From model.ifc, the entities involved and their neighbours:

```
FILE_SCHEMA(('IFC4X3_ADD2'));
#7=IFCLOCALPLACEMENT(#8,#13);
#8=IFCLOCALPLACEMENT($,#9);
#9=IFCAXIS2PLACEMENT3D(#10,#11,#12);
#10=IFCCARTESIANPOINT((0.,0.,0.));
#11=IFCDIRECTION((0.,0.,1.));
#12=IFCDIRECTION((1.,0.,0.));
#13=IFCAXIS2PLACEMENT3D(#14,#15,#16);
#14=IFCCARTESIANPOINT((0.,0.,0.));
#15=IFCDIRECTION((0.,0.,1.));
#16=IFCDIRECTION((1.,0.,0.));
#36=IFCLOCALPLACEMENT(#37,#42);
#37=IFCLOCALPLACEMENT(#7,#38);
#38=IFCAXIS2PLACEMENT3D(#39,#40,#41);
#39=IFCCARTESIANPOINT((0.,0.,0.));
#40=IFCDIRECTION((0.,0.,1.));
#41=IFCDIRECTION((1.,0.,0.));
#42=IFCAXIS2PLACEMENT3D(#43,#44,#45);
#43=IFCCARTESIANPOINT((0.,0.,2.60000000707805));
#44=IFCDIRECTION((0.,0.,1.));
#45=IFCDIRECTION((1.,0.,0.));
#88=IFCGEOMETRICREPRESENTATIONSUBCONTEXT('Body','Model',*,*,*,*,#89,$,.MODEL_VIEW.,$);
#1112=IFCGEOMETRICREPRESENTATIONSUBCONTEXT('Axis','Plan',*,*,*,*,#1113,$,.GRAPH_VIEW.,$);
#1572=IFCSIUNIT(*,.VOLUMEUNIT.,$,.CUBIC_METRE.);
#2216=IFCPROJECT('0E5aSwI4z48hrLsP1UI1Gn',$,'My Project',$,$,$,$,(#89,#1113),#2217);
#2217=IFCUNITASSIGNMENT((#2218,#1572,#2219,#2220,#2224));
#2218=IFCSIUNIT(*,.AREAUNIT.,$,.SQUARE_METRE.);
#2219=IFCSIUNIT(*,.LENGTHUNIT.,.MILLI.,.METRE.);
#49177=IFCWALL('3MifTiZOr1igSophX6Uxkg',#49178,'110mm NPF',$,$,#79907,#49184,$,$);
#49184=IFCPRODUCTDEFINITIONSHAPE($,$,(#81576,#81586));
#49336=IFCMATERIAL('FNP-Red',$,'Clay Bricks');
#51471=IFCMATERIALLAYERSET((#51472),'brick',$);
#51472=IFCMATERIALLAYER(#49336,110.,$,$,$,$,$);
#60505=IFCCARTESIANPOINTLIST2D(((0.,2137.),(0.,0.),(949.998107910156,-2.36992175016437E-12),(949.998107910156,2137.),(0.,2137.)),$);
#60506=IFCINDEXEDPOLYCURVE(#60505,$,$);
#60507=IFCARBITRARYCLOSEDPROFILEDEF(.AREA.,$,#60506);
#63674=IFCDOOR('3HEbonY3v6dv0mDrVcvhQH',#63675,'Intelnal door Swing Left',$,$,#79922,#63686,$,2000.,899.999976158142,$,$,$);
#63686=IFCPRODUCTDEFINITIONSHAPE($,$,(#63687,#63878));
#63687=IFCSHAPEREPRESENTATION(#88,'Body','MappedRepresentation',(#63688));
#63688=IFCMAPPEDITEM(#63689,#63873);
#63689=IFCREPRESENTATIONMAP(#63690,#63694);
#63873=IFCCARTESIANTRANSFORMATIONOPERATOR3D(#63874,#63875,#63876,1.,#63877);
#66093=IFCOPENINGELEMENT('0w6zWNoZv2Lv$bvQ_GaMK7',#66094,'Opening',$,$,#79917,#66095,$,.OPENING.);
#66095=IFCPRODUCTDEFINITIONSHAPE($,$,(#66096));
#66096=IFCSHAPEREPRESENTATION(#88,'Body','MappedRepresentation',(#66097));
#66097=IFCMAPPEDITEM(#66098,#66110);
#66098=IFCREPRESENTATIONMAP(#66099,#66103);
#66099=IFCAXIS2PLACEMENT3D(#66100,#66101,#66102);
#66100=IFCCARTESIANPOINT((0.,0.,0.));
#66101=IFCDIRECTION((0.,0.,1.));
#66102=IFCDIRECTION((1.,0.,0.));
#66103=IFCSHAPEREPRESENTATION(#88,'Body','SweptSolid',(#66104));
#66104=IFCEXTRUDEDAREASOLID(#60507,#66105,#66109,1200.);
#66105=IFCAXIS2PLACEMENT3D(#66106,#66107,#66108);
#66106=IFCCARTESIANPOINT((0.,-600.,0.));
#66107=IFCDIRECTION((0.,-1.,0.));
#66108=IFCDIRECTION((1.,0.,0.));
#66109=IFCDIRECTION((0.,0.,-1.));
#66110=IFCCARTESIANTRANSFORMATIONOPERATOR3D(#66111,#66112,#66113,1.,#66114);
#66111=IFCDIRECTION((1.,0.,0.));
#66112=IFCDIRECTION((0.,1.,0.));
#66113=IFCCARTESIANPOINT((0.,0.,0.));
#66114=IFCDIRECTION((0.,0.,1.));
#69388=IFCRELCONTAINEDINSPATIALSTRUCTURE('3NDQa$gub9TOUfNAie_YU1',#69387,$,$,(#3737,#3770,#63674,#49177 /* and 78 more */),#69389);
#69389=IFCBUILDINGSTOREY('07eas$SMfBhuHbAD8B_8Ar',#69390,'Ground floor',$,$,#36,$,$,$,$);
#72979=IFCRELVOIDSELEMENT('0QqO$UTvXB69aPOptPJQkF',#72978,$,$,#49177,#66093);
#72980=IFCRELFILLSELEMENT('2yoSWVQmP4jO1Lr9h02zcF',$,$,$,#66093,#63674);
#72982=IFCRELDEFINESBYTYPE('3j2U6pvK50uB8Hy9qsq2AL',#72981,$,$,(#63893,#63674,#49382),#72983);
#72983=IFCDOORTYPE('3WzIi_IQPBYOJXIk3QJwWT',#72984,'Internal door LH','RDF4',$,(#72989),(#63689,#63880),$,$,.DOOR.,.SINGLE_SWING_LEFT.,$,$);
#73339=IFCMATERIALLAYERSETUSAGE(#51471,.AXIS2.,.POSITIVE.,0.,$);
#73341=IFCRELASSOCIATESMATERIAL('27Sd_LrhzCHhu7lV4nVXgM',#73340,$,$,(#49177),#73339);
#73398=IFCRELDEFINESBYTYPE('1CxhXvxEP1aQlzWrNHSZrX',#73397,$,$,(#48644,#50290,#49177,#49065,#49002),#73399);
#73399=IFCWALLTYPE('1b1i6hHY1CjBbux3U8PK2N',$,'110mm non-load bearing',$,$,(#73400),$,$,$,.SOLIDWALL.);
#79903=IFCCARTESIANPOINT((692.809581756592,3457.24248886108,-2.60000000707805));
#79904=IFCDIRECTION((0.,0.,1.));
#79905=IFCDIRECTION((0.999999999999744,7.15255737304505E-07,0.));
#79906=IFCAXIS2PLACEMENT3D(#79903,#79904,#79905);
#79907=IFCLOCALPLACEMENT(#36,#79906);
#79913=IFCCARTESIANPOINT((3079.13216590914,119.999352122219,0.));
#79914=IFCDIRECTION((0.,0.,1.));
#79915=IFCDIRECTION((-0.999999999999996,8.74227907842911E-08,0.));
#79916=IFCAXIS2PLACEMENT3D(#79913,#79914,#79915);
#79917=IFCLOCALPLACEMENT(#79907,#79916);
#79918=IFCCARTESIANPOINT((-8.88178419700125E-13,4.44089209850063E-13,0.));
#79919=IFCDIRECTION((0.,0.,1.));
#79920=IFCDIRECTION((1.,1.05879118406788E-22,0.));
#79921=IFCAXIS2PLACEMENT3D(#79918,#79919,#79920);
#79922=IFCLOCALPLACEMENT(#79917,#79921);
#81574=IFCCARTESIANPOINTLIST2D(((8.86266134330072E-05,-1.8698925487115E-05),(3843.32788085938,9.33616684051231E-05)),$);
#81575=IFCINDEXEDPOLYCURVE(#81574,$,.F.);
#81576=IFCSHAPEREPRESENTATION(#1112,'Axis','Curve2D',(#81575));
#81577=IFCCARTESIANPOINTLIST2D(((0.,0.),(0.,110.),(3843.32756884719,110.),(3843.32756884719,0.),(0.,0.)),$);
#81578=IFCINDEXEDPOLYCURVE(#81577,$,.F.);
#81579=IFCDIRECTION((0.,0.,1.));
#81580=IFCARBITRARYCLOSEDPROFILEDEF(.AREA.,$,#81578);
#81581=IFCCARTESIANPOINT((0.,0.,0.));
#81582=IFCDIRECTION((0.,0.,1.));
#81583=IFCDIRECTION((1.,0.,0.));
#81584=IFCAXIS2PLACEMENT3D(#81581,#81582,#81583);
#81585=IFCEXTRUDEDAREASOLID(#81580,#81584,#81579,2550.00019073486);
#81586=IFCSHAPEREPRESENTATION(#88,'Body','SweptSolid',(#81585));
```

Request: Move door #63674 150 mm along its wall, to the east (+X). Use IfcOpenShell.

```python
import ifcopenshell
import ifcopenshell.api.geometry
import ifcopenshell.util.placement
import ifcopenshell.util.unit

model = ifcopenshell.open("model.ifc")
unit_scale = ifcopenshell.util.unit.calculate_unit_scale(model)

door = model.by_guid("3HEbonY3v6dv0mDrVcvhQH")
opening = door.FillsVoids[0].RelatingOpeningElement
wall = opening.VoidsElements[0].RelatingBuildingElement

wall_matrix = ifcopenshell.util.placement.get_local_placement(wall.ObjectPlacement)
shift = wall_matrix[:3, 0] * 0.15 / unit_scale
before = ifcopenshell.util.placement.get_local_placement(door.ObjectPlacement)[:3, 3].copy()

# The door is placed relative to its opening, so it follows when the opening moves.
matrix = ifcopenshell.util.placement.get_local_placement(opening.ObjectPlacement)
matrix[:3, 3] += shift
ifcopenshell.api.geometry.edit_object_placement(
    model, product=opening, matrix=matrix, is_si=False, should_transform_children=True
)

after = ifcopenshell.util.placement.get_local_placement(door.ObjectPlacement)[:3, 3]
print("door moved by", (after - before).round(3) + 0.0)

model.write("model_edited.ifc")
```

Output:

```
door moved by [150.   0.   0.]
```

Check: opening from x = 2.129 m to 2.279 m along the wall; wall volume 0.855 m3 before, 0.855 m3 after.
